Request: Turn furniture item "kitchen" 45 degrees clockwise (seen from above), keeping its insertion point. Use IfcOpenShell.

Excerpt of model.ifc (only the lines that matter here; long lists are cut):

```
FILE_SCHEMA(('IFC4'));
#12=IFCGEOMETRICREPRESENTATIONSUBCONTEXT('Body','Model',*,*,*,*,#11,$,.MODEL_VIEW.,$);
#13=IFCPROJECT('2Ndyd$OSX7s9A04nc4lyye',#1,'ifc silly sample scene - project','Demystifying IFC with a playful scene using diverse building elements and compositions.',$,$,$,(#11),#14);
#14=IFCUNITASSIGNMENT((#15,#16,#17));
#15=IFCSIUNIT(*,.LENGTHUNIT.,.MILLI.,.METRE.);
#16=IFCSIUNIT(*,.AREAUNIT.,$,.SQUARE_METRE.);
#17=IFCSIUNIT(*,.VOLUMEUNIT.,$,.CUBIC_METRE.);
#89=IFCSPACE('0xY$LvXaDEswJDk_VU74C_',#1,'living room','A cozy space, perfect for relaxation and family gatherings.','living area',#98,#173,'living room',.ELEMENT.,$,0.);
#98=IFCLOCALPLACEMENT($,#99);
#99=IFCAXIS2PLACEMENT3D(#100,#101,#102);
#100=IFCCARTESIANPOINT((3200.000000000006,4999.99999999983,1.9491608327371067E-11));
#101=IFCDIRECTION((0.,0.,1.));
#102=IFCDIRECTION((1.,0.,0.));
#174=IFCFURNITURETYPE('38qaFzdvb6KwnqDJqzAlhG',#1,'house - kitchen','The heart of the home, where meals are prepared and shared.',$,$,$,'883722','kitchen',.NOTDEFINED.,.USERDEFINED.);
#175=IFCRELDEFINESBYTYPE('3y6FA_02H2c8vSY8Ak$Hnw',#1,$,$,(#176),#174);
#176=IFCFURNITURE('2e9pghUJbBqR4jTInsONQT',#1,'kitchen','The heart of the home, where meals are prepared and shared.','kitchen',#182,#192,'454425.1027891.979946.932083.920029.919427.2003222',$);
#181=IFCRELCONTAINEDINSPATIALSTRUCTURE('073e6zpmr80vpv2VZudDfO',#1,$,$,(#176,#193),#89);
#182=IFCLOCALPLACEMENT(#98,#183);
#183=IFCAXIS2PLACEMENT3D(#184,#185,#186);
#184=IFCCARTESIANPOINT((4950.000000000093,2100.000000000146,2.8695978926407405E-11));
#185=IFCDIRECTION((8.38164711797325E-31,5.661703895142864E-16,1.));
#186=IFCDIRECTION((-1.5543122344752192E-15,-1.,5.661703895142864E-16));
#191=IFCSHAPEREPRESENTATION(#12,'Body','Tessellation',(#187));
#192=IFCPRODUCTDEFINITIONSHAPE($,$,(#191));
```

```python
import ifcopenshell
import ifcopenshell.api.geometry
import ifcopenshell.util.placement

model = ifcopenshell.open("model.ifc")

item = model.by_guid("2e9pghUJbBqR4jTInsONQT")
matrix = ifcopenshell.util.placement.get_local_placement(item.ObjectPlacement)
matrix = matrix @ ifcopenshell.util.placement.rotation(-45, "Z")
ifcopenshell.api.geometry.edit_object_placement(model, product=item, matrix=matrix, is_si=False)

print(ifcopenshell.util.placement.get_local_placement(item.ObjectPlacement).round(3) + 0.0)

model.write("model_edited.ifc")
```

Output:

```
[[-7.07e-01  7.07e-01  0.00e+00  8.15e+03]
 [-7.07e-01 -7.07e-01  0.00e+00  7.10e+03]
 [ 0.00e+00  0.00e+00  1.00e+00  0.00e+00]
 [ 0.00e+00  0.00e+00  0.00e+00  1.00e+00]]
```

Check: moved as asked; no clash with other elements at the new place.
